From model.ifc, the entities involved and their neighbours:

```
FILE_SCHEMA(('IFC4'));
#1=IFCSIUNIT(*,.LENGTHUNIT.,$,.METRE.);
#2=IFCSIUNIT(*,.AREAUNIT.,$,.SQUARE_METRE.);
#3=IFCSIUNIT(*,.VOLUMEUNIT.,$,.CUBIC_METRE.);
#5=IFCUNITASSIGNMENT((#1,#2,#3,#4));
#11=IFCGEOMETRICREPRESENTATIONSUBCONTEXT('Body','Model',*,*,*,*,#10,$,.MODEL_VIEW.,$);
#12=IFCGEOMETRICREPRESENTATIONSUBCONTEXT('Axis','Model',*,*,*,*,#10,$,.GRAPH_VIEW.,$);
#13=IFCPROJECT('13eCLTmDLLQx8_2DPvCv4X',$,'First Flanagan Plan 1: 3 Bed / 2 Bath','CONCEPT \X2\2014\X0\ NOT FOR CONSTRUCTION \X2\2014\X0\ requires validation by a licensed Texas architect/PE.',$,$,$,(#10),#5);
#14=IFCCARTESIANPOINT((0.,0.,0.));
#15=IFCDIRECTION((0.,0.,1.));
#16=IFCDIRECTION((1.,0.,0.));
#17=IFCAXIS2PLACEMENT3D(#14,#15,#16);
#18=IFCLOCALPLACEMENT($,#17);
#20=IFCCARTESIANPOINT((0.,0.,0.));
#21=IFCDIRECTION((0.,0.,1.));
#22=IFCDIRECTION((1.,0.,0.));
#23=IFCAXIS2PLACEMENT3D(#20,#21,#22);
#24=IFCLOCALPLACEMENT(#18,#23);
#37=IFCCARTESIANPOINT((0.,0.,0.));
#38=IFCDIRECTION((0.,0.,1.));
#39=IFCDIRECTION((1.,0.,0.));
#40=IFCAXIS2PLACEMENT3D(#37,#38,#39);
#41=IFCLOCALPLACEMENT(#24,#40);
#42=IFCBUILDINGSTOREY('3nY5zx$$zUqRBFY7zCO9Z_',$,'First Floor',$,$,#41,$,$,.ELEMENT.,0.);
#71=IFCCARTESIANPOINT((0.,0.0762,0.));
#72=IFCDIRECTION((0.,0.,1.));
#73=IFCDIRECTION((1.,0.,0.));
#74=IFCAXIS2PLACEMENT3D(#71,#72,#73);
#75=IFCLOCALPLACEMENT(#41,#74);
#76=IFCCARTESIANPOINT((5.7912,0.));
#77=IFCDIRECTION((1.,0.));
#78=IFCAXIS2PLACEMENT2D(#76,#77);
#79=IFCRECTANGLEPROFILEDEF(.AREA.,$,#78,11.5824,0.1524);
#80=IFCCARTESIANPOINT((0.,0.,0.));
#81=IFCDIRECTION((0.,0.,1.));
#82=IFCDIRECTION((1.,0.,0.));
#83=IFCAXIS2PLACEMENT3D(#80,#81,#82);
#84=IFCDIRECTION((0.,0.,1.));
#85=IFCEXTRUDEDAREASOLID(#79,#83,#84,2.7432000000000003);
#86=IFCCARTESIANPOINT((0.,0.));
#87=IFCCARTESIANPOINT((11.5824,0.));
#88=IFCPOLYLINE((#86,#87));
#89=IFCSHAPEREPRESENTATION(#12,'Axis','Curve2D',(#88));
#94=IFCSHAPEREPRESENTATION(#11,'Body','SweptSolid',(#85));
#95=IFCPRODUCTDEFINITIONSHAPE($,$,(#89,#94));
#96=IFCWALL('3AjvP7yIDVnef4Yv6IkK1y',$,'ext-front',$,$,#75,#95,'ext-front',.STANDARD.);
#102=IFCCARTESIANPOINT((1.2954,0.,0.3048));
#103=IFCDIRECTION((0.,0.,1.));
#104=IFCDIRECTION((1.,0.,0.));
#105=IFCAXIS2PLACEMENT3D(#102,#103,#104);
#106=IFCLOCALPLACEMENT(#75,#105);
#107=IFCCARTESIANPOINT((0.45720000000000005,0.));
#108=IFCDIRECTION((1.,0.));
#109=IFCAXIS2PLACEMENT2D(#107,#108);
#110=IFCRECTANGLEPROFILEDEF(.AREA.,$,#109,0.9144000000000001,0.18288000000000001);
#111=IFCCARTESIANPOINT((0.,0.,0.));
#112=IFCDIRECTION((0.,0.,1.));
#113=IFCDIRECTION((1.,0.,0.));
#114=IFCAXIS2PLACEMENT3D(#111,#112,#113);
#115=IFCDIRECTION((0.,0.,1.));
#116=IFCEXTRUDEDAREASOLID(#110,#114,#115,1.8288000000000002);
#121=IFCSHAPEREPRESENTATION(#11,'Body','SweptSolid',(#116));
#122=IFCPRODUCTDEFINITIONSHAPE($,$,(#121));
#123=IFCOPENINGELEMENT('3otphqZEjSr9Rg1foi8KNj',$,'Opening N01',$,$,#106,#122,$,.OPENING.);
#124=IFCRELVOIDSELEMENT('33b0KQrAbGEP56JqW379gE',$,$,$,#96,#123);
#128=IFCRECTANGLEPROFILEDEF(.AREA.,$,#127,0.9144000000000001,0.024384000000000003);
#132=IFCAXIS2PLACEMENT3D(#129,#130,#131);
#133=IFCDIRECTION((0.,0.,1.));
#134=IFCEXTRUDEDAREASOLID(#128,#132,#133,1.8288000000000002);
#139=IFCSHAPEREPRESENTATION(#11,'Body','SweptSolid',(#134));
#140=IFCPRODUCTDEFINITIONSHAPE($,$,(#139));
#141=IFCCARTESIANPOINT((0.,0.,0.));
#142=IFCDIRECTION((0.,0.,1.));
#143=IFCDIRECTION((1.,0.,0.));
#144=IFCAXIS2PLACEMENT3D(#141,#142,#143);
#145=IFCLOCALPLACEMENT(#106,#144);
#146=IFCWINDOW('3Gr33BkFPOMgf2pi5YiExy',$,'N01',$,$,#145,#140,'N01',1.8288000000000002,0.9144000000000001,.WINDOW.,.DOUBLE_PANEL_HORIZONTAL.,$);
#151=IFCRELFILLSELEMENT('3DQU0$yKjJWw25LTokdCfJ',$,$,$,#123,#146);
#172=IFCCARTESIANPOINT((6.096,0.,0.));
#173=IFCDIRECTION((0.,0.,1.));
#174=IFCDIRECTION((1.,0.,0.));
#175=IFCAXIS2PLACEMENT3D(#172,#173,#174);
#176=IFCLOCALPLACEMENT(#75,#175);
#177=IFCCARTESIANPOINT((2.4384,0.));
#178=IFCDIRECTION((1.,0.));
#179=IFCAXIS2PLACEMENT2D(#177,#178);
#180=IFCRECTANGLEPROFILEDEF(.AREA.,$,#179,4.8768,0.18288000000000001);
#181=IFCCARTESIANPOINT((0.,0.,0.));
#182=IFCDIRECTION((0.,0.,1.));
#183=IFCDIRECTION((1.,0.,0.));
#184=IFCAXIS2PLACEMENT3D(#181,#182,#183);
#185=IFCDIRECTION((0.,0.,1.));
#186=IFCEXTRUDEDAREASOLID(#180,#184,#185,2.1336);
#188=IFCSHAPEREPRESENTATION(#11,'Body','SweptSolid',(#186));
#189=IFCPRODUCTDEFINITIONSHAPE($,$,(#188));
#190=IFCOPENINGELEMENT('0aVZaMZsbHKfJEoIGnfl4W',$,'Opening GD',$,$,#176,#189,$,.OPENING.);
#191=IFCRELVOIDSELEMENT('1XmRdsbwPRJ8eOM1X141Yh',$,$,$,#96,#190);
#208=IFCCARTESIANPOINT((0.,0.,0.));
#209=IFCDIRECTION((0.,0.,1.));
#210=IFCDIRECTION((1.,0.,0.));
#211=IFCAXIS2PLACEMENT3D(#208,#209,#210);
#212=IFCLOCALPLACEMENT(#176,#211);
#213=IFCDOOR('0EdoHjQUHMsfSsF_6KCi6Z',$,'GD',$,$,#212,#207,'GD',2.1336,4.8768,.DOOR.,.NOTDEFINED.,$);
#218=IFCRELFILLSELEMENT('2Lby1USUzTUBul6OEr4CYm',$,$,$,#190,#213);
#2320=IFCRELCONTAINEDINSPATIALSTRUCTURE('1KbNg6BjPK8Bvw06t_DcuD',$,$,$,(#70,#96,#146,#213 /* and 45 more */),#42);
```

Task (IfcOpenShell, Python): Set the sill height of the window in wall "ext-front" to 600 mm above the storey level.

```python
import numpy as np
import ifcopenshell
import ifcopenshell.api.geometry
import ifcopenshell.geom
import ifcopenshell.util.element
import ifcopenshell.util.placement
import ifcopenshell.util.shape
import ifcopenshell.util.unit

model = ifcopenshell.open("model.ifc")
unit_scale = ifcopenshell.util.unit.calculate_unit_scale(model)

window = model.by_guid("3Gr33BkFPOMgf2pi5YiExy")
opening = window.FillsVoids[0].RelatingOpeningElement
storey = ifcopenshell.util.element.get_container(window, ifc_class="IfcBuildingStorey")
level = ifcopenshell.util.placement.get_local_placement(storey.ObjectPlacement)[2, 3]

# The opening's origin need not be at the sill, so measure its lowest point.
shape = ifcopenshell.geom.create_shape(ifcopenshell.geom.settings(), opening)
bottom = ifcopenshell.util.shape.get_shape_bottom_elevation(shape, shape.geometry) / unit_scale
dz = level + 0.6 / unit_scale - bottom

shift = np.array([0.0, 0.0, dz])
# The window is placed relative to its opening, so it follows when the opening moves.
matrix = ifcopenshell.util.placement.get_local_placement(opening.ObjectPlacement)
matrix[:3, 3] += shift
ifcopenshell.api.geometry.edit_object_placement(
    model, product=opening, matrix=matrix, is_si=False, should_transform_children=True
)

print(f"moved by {dz * unit_scale:+.3f} m")

model.write("model_updated.ifc")
```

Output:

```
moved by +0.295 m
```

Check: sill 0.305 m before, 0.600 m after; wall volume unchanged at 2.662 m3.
